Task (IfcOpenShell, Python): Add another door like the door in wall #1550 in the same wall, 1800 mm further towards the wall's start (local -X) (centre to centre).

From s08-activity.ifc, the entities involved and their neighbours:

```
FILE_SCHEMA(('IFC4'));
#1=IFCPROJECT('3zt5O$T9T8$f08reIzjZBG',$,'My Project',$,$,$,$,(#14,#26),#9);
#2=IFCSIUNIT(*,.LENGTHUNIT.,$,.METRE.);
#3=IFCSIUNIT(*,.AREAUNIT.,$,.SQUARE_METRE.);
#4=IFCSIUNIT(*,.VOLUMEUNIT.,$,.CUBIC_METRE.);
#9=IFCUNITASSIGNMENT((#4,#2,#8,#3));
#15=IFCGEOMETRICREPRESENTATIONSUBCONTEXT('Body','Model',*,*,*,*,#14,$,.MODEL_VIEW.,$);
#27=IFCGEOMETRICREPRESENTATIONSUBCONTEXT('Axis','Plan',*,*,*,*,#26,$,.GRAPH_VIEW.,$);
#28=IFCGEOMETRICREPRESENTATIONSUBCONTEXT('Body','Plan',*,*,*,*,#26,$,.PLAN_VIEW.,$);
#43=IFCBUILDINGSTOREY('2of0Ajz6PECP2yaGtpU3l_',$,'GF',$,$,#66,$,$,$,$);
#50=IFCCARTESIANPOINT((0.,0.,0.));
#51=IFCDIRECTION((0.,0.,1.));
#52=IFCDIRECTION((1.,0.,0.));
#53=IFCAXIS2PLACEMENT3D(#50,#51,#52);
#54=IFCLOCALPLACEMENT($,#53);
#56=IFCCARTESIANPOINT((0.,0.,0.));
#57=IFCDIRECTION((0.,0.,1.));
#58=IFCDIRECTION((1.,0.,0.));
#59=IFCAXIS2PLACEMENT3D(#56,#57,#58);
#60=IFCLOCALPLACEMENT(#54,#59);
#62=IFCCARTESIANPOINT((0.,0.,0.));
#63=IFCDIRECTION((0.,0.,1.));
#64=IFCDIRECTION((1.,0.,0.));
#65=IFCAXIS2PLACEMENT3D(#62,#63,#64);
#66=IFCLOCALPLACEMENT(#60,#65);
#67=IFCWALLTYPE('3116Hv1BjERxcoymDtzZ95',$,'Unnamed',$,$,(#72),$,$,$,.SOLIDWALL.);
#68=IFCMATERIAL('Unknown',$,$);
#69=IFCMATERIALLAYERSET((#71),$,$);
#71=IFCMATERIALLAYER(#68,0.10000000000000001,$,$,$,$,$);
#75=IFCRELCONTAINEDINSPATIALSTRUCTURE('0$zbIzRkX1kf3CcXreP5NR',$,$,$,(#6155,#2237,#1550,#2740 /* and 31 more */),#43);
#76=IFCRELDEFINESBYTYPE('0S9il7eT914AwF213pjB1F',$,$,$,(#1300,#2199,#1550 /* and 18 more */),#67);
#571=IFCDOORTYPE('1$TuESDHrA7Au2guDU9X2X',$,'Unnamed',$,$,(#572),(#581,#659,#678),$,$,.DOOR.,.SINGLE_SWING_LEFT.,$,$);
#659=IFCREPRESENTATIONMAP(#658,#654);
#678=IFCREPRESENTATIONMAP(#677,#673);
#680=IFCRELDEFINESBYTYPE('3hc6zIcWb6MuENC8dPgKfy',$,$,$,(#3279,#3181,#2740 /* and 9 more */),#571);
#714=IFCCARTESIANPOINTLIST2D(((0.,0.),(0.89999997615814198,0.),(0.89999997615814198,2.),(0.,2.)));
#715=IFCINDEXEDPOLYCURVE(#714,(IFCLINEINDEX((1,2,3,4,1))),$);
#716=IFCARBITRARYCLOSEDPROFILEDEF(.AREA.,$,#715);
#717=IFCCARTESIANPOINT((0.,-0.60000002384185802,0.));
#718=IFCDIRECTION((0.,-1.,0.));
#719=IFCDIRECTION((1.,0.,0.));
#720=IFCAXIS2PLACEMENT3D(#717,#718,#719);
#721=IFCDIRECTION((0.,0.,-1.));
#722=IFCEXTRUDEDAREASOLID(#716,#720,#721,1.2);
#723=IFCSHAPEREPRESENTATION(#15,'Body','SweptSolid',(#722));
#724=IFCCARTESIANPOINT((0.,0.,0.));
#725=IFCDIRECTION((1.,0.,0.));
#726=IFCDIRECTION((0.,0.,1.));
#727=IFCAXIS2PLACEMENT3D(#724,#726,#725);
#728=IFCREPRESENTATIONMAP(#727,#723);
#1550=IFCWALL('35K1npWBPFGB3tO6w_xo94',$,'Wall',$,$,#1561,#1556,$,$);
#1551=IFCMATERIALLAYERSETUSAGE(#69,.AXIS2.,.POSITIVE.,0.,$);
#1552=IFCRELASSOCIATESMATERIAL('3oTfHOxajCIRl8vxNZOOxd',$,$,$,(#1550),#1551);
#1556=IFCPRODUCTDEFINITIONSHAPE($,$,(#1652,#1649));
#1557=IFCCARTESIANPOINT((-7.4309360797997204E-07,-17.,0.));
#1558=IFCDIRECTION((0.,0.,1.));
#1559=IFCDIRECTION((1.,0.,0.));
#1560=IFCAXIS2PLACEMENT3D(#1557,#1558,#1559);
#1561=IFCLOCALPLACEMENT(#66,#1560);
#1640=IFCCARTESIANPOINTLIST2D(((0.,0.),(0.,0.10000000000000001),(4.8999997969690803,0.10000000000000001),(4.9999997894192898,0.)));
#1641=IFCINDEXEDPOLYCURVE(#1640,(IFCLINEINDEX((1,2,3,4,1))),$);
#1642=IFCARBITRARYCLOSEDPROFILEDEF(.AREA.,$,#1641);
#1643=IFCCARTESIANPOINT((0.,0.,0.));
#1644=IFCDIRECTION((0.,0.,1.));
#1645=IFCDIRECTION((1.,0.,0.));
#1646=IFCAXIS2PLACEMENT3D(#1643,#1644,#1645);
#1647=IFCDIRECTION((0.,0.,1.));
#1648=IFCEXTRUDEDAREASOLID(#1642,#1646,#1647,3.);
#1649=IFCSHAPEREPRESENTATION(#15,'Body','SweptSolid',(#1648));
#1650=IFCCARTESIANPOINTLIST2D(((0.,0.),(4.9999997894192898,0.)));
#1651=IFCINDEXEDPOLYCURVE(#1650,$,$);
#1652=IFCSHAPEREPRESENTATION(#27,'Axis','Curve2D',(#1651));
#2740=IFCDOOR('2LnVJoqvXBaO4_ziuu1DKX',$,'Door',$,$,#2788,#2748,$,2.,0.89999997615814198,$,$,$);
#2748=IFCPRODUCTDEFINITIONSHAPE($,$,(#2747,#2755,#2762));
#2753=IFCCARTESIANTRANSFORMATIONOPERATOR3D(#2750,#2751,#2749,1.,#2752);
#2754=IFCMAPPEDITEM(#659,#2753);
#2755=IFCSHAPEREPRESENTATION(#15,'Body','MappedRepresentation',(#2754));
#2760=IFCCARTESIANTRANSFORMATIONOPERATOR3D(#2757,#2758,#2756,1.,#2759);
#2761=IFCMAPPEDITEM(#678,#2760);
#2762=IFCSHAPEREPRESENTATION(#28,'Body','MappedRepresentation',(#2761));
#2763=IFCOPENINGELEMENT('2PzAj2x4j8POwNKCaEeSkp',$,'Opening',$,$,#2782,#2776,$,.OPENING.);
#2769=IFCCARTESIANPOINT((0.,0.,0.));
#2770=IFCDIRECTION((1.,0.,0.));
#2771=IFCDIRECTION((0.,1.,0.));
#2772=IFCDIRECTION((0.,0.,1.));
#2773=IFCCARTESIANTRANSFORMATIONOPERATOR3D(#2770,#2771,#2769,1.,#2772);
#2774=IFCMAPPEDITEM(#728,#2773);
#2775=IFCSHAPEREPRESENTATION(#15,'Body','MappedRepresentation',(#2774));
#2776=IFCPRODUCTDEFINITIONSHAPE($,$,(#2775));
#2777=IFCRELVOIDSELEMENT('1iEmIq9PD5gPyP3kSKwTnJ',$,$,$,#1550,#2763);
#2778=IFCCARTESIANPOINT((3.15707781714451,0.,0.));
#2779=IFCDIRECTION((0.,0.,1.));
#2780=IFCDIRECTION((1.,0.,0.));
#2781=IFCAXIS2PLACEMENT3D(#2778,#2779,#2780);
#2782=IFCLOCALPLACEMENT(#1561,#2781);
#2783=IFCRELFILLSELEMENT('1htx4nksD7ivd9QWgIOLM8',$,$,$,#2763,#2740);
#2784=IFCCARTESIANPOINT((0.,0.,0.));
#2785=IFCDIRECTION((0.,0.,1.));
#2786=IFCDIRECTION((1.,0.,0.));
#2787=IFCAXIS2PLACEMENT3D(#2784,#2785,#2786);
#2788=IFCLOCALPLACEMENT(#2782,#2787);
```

```python
import ifcopenshell
import ifcopenshell.api.feature
import ifcopenshell.api.geometry
import ifcopenshell.api.root
import ifcopenshell.geom
import ifcopenshell.util.element
import ifcopenshell.util.placement
import ifcopenshell.util.shape
import ifcopenshell.util.unit

model = ifcopenshell.open("s08-activity.ifc")
unit_scale = ifcopenshell.util.unit.calculate_unit_scale(model)
settings = ifcopenshell.geom.settings()


def volume(element):
    """Net volume in cubic metres, openings subtracted."""
    shape = ifcopenshell.geom.create_shape(settings, element)
    return ifcopenshell.util.shape.get_volume(shape.geometry)


door = model.by_guid("2LnVJoqvXBaO4_ziuu1DKX")
opening = door.FillsVoids[0].RelatingOpeningElement
wall = opening.VoidsElements[0].RelatingBuildingElement
before = volume(wall)
shift = ifcopenshell.util.placement.get_local_placement(wall.ObjectPlacement)[:3, 0] * -1.8 / unit_scale

# copy_class copies the void relationship, type, container and properties, but no geometry.
new_opening = ifcopenshell.api.root.copy_class(model, product=opening)
new_opening.Representation = ifcopenshell.util.element.copy_deep(
    model, opening.Representation, exclude=["IfcGeometricRepresentationContext", "IfcRepresentationMap"]
)
new_door = ifcopenshell.api.root.copy_class(model, product=door)
new_door.Representation = ifcopenshell.util.element.copy_deep(
    model, door.Representation, exclude=["IfcGeometricRepresentationContext", "IfcRepresentationMap"]
)
ifcopenshell.api.feature.add_filling(model, opening=new_opening, element=new_door)

for old, new in ((opening, new_opening), (door, new_door)):
    matrix = ifcopenshell.util.placement.get_local_placement(old.ObjectPlacement)
    matrix[:3, 3] += shift
    ifcopenshell.api.geometry.edit_object_placement(model, product=new, matrix=matrix, is_si=False)

after = volume(wall)

print(f"wall volume {before:.3f} -> {after:.3f} m3")

model.write("s08-activity-out.ifc")
```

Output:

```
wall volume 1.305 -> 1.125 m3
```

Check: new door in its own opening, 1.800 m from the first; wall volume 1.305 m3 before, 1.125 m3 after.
